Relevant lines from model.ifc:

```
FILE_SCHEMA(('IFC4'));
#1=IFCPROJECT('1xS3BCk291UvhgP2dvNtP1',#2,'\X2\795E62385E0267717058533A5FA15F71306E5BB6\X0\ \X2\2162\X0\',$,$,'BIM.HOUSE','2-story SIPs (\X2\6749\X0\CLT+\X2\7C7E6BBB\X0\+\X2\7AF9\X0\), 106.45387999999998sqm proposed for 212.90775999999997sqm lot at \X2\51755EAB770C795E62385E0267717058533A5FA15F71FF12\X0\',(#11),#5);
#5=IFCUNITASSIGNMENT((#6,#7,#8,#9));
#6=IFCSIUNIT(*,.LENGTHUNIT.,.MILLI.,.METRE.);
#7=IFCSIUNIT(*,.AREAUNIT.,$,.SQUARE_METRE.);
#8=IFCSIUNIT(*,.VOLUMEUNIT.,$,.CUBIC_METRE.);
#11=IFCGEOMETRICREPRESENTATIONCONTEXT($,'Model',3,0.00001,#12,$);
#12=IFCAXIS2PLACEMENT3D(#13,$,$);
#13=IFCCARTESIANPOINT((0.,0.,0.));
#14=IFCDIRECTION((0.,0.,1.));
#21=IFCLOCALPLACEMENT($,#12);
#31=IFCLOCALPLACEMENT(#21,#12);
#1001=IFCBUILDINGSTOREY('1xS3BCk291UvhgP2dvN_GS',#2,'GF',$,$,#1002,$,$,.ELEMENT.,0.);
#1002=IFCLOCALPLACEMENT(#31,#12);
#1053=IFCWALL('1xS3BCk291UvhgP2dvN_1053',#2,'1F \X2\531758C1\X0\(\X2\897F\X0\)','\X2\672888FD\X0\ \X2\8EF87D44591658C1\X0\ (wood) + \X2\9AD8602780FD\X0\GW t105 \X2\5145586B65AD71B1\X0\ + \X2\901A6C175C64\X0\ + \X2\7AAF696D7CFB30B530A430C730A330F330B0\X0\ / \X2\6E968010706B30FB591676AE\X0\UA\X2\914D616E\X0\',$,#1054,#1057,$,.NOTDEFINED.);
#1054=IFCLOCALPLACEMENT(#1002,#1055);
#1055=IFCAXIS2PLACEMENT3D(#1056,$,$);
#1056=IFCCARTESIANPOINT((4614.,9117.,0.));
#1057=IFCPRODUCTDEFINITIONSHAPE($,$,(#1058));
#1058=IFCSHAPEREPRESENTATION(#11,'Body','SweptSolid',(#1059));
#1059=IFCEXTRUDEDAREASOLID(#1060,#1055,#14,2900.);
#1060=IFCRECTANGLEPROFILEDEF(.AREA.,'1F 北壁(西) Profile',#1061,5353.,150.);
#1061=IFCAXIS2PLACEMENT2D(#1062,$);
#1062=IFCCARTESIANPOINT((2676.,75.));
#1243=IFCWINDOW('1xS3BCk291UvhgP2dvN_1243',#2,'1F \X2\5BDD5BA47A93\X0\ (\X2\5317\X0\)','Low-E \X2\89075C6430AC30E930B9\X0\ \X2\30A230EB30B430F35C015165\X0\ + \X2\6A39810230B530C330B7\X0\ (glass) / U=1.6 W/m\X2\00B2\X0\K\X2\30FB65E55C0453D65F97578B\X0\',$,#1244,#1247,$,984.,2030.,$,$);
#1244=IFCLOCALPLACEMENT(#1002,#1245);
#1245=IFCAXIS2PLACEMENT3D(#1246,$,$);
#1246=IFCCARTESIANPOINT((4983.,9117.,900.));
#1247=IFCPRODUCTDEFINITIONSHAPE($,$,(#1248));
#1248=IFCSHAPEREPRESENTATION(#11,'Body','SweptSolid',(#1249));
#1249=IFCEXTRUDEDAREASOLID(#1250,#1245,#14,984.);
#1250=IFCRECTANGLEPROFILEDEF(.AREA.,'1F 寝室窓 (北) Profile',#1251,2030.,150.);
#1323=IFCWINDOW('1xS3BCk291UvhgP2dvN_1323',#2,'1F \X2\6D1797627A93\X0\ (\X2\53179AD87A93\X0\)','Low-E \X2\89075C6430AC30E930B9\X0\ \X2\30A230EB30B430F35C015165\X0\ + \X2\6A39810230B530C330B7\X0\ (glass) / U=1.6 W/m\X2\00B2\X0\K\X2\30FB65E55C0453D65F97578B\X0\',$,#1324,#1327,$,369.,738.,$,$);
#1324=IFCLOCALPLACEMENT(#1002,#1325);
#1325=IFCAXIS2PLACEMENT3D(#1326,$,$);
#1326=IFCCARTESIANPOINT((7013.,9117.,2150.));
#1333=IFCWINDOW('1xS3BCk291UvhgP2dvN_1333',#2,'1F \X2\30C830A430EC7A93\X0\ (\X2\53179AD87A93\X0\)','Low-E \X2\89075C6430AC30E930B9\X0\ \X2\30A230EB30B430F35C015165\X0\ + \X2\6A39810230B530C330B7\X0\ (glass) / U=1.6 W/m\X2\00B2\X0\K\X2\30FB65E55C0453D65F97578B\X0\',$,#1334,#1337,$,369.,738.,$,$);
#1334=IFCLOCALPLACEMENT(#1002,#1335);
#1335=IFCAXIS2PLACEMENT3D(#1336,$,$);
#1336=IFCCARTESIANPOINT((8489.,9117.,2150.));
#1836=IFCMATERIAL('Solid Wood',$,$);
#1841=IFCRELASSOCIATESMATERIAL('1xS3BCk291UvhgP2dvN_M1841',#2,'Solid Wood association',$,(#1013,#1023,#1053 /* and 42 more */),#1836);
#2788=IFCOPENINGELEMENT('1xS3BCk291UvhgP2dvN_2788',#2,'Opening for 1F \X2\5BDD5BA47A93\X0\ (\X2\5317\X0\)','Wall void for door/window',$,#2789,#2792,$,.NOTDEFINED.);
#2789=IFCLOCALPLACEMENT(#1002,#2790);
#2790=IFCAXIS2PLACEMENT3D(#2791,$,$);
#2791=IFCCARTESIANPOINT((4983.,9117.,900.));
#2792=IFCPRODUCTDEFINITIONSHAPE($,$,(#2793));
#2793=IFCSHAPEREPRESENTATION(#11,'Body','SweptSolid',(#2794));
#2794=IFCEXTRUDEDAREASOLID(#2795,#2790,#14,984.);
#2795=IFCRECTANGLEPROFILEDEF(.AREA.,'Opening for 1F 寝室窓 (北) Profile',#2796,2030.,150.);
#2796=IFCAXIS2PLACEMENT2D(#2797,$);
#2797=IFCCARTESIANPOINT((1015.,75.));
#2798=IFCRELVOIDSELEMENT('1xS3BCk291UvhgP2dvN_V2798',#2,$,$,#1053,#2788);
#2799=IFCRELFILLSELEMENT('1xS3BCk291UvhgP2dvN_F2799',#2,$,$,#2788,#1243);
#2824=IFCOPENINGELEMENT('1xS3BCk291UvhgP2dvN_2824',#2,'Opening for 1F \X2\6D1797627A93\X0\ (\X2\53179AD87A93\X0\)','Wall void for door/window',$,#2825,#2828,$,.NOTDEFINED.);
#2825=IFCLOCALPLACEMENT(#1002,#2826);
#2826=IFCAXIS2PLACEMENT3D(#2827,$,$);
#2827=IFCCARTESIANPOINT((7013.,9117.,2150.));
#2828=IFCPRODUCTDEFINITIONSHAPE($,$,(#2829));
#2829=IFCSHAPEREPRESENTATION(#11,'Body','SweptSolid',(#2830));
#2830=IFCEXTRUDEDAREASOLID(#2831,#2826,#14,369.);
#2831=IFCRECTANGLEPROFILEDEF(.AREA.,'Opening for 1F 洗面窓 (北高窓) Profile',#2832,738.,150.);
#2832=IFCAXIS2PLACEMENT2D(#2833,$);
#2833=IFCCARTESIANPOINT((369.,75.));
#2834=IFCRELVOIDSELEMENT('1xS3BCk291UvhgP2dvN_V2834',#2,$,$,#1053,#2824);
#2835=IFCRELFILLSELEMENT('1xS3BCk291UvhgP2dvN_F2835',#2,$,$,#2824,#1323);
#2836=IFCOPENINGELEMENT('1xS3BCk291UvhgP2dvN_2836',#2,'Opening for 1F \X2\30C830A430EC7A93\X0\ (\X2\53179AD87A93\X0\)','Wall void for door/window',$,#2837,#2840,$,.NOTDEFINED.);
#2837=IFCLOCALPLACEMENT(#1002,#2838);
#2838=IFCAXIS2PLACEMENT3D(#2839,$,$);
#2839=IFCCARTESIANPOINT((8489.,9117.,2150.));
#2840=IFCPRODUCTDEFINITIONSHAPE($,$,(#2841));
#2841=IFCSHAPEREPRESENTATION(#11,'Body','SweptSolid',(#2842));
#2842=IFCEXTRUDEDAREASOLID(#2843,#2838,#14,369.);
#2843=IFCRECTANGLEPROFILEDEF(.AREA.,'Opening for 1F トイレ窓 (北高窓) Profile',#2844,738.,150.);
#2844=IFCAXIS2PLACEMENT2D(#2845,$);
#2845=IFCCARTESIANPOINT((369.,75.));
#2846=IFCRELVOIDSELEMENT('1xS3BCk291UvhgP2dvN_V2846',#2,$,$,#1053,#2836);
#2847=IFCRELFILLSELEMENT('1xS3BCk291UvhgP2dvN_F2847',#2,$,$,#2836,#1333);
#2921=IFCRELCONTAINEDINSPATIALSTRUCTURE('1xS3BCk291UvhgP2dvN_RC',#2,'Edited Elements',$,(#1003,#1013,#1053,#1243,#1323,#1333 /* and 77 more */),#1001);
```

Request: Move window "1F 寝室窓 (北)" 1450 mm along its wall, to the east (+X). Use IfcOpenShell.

```python
import ifcopenshell
import ifcopenshell.api.geometry
import ifcopenshell.util.placement
import ifcopenshell.util.unit

model = ifcopenshell.open("model.ifc")
unit_scale = ifcopenshell.util.unit.calculate_unit_scale(model)

window = model.by_id(1243)
opening = window.FillsVoids[0].RelatingOpeningElement
wall = opening.VoidsElements[0].RelatingBuildingElement

wall_matrix = ifcopenshell.util.placement.get_local_placement(wall.ObjectPlacement)
shift = wall_matrix[:3, 0] * 1.45 / unit_scale
before = ifcopenshell.util.placement.get_local_placement(window.ObjectPlacement)[:3, 3].copy()

# The window is not placed relative to its opening, so move both.
for product in (opening, window):
    matrix = ifcopenshell.util.placement.get_local_placement(product.ObjectPlacement)
    matrix[:3, 3] += shift
    ifcopenshell.api.geometry.edit_object_placement(model, product=product, matrix=matrix, is_si=False)

after = ifcopenshell.util.placement.get_local_placement(window.ObjectPlacement)[:3, 3]
print("window moved by", (after - before).round(3) + 0.0)

model.write("model_updated.ifc")
```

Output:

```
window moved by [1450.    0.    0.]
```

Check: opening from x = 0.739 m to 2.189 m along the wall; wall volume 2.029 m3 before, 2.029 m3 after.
